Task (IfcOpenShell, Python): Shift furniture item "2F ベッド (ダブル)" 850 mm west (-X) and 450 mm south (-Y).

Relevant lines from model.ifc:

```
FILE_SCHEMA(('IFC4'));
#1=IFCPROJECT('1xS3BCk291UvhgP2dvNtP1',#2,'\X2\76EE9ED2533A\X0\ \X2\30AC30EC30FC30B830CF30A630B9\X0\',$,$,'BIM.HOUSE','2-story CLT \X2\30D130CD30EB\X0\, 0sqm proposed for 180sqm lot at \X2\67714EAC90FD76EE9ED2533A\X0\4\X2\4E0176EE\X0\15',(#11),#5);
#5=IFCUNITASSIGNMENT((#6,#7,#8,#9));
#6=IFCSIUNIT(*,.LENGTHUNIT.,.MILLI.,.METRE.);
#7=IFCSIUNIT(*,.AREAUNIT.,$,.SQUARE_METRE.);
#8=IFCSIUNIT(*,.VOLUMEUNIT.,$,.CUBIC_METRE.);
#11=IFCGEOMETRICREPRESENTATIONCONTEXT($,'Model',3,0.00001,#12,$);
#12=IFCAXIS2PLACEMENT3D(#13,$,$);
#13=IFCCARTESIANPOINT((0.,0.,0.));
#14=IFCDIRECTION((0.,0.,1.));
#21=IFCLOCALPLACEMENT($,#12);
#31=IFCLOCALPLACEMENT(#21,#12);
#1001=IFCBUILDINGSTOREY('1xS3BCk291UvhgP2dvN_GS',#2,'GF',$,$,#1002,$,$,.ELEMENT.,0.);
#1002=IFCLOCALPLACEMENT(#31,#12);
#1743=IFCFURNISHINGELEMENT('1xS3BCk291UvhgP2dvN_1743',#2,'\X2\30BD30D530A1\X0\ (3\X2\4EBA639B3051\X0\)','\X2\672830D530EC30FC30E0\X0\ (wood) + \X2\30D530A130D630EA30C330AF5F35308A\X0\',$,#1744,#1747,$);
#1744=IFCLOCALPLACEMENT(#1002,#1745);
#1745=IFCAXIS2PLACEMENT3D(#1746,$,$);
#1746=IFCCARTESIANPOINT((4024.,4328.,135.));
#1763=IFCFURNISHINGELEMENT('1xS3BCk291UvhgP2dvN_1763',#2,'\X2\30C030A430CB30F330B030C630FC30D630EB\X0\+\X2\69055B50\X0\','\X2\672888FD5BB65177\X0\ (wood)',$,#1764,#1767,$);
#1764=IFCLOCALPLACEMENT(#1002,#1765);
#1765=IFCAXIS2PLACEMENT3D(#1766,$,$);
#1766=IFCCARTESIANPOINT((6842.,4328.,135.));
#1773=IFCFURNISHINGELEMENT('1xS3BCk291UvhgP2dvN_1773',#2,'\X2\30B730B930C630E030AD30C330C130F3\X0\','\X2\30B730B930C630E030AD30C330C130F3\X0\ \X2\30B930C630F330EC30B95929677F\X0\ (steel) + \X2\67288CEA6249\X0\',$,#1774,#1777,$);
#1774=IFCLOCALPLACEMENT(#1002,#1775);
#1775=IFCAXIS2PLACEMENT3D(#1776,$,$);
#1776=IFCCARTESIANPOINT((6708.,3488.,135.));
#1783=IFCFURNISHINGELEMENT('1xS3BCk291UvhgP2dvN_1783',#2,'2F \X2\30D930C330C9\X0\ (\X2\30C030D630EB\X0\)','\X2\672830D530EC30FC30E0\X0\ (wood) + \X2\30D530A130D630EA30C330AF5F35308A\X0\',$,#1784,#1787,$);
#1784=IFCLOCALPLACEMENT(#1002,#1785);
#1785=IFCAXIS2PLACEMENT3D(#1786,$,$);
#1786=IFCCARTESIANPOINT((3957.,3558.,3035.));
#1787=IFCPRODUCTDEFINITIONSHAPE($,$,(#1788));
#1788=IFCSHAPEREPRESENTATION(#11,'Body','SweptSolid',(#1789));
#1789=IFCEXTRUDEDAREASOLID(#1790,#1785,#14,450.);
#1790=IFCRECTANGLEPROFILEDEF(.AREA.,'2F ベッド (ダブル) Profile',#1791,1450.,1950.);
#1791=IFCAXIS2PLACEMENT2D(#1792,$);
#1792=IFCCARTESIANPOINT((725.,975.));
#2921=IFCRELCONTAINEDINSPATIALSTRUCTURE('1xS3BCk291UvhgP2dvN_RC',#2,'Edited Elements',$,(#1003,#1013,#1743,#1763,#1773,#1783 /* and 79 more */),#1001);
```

```python
import ifcopenshell
import ifcopenshell.api.geometry
import ifcopenshell.util.placement
import ifcopenshell.util.unit

model = ifcopenshell.open("model.ifc")
unit_scale = ifcopenshell.util.unit.calculate_unit_scale(model)

item = model.by_guid("1xS3BCk291UvhgP2dvN_1783")
matrix = ifcopenshell.util.placement.get_local_placement(item.ObjectPlacement)
matrix[0, 3] -= 0.85 / unit_scale
matrix[1, 3] -= 0.45 / unit_scale
ifcopenshell.api.geometry.edit_object_placement(model, product=item, matrix=matrix, is_si=False)

print(ifcopenshell.util.placement.get_local_placement(item.ObjectPlacement).round(3) + 0.0)

model.write("model_updated.ifc")
```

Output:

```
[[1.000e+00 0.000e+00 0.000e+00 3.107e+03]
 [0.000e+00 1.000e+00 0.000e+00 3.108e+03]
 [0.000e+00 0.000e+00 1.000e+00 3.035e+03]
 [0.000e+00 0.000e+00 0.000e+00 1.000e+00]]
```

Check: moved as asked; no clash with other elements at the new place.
